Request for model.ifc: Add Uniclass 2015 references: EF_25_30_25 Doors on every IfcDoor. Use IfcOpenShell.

First a look at what the model holds.

```python
import ifcopenshell

model = ifcopenshell.open("model.ifc")
print(model.schema)
print("classifications:", [c.Name for c in model.by_type("IfcClassification")])
for ifc_class in ("IfcDoor", "IfcRoof", "IfcStair", "IfcWall", "IfcWindow"):
    print(ifc_class, len(model.by_type(ifc_class)))
```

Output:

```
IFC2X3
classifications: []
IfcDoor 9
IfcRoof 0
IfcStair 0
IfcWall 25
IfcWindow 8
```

```python
import ifcopenshell
import ifcopenshell.api.classification

model = ifcopenshell.open("model.ifc")

# IFC2X3 requires Source and Edition and has no link from the project to the system.
system = model.create_entity("IfcClassification", Source="NBS", Edition="2015", Name="Uniclass 2015")

codes = {
    "IfcDoor": ("EF_25_30_25", "Doors"),
}
for ifc_class, (code, name) in codes.items():
    products = model.by_type(ifc_class)
    ifcopenshell.api.classification.add_reference(
        model, products=products, classification=system, identification=code, name=name
    )
    print(code, len(products))

model.write("model-out.ifc")
```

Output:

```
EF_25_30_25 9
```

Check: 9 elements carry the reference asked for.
